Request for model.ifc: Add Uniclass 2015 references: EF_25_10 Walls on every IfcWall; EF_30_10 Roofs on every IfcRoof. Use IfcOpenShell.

First a look at what the model holds.

```python
import ifcopenshell

model = ifcopenshell.open("model.ifc")
print(model.schema)
print("classifications:", [c.Name for c in model.by_type("IfcClassification")])
for ifc_class in ("IfcDoor", "IfcRoof", "IfcStair", "IfcWall", "IfcWindow"):
    print(ifc_class, len(model.by_type(ifc_class)))
```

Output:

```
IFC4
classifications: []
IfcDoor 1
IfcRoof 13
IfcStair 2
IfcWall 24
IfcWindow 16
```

```python
import ifcopenshell
import ifcopenshell.api.classification

model = ifcopenshell.open("model.ifc")

system = ifcopenshell.api.classification.add_classification(model, classification="Uniclass 2015")

codes = {
    "IfcWall": ("EF_25_10", "Walls"),
    "IfcRoof": ("EF_30_10", "Roofs"),
}
for ifc_class, (code, name) in codes.items():
    products = model.by_type(ifc_class)
    ifcopenshell.api.classification.add_reference(
        model, products=products, classification=system, identification=code, name=name
    )
    print(code, len(products))

model.write("model_v2.ifc")
```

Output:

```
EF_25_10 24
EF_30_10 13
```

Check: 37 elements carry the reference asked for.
